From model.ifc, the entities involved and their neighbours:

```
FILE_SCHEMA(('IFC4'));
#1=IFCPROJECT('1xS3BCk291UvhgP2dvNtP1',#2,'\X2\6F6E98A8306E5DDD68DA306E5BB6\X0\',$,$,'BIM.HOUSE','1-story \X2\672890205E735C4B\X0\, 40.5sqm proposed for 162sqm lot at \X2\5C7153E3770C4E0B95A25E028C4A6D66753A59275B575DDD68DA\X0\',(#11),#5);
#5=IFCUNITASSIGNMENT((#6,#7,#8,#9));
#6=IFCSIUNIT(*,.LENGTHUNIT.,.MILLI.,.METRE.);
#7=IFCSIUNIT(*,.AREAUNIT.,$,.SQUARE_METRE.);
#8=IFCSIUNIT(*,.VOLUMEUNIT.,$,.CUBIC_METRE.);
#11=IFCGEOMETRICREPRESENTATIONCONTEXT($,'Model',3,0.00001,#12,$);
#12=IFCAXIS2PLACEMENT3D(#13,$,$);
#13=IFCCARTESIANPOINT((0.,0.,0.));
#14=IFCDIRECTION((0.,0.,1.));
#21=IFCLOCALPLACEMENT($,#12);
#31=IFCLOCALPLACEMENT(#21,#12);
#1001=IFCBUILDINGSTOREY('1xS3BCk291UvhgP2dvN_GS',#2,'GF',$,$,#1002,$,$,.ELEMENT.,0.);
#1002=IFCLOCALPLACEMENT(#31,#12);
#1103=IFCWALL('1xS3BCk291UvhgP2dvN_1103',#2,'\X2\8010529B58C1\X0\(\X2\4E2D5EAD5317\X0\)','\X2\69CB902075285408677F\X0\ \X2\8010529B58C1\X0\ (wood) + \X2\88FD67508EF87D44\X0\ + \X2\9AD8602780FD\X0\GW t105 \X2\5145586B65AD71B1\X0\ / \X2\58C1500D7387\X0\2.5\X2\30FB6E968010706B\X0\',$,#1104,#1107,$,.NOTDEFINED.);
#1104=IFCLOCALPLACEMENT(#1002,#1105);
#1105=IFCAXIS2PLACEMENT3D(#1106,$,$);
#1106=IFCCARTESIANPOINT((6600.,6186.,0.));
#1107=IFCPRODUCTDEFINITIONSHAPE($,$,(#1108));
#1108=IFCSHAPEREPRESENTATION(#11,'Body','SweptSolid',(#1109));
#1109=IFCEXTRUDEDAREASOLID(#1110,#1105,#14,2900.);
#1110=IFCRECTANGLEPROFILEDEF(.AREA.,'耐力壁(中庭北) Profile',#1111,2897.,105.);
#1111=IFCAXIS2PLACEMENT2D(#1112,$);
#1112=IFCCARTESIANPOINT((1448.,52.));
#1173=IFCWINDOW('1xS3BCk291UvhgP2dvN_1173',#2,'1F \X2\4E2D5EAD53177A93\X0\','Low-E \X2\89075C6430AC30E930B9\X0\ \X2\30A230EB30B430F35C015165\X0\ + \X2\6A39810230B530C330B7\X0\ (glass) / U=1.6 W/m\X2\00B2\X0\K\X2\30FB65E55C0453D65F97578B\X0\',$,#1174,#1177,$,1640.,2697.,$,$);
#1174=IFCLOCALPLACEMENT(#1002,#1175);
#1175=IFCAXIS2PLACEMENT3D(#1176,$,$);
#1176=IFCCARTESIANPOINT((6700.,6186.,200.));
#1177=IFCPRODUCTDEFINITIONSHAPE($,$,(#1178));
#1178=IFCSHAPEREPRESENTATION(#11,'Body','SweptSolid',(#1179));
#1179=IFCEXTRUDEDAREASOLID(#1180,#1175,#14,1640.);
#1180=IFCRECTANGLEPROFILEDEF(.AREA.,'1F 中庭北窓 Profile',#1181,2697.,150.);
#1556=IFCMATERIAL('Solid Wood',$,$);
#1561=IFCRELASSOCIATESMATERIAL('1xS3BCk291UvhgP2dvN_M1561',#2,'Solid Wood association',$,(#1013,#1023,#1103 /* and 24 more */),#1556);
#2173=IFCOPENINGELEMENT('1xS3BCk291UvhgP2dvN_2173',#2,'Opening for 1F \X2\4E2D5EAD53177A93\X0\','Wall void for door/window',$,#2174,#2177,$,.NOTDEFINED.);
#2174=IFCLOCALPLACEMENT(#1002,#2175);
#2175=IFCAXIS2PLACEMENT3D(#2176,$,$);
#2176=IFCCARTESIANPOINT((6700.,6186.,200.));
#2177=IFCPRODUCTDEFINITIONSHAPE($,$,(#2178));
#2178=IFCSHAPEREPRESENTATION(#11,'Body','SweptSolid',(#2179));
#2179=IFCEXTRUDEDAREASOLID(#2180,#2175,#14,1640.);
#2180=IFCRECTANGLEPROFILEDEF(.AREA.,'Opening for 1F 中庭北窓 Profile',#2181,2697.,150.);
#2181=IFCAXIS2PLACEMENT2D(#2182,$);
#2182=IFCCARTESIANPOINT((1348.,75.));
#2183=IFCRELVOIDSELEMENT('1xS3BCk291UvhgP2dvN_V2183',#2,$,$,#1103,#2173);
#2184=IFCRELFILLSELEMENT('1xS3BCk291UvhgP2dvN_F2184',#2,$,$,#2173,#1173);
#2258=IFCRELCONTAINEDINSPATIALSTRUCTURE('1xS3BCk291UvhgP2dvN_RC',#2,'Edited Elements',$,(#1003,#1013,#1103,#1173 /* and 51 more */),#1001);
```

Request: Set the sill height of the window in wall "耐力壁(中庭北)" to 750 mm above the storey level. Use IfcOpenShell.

```python
import numpy as np
import ifcopenshell
import ifcopenshell.api.geometry
import ifcopenshell.geom
import ifcopenshell.util.element
import ifcopenshell.util.placement
import ifcopenshell.util.shape
import ifcopenshell.util.unit

model = ifcopenshell.open("model.ifc")
unit_scale = ifcopenshell.util.unit.calculate_unit_scale(model)

window = model.by_guid("1xS3BCk291UvhgP2dvN_1173")
opening = window.FillsVoids[0].RelatingOpeningElement
storey = ifcopenshell.util.element.get_container(window, ifc_class="IfcBuildingStorey")
level = ifcopenshell.util.placement.get_local_placement(storey.ObjectPlacement)[2, 3]

# The opening's origin need not be at the sill, so measure its lowest point.
shape = ifcopenshell.geom.create_shape(ifcopenshell.geom.settings(), opening)
bottom = ifcopenshell.util.shape.get_shape_bottom_elevation(shape, shape.geometry) / unit_scale
dz = level + 0.75 / unit_scale - bottom

shift = np.array([0.0, 0.0, dz])
# The window is not placed relative to its opening, so move both.
for product in (opening, window):
    matrix = ifcopenshell.util.placement.get_local_placement(product.ObjectPlacement)
    matrix[:3, 3] += shift
    ifcopenshell.api.geometry.edit_object_placement(model, product=product, matrix=matrix, is_si=False)

print(f"moved by {dz * unit_scale:+.3f} m")

model.write("model_rev.ifc")
```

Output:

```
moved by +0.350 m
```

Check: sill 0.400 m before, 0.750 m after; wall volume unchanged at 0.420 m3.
